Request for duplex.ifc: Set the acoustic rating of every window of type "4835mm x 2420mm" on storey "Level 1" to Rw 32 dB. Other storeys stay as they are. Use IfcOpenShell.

First a look at what the model holds.

```python
import ifcopenshell
import ifcopenshell.util.element

model = ifcopenshell.open("duplex.ifc")
print(model.schema)
storey = next(s for s in model.by_type("IfcBuildingStorey") if s.Name == "Level 1")
windows = [e for e in ifcopenshell.util.element.get_decomposition(storey) if e.is_a("IfcWindow")]
seen = {}
for e in windows:
    element_type = ifcopenshell.util.element.get_type(e)
    key = (element_type.Name if element_type != e and element_type else None, ifcopenshell.util.element.get_pset(e, "Pset_WindowCommon", "AcousticRating"))
    seen[key] = seen.get(key, 0) + 1
for (name, value), count in sorted(seen.items(), key=str):
    print(count, "x", name, "|", value)
```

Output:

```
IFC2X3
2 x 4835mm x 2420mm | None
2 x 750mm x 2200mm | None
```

```python
import ifcopenshell
import ifcopenshell.api.pset
import ifcopenshell.util.element

model = ifcopenshell.open("duplex.ifc")

storey = next(s for s in model.by_type("IfcBuildingStorey") if s.Name == "Level 1")
windows = [e for e in ifcopenshell.util.element.get_decomposition(storey) if e.is_a("IfcWindow")]

count = 0
for e in windows:
    element_type = ifcopenshell.util.element.get_type(e)
    if element_type in (None, e) or element_type.Name != "4835mm x 2420mm":
        continue
    # add_pset returns the element's existing set when there is one.
    pset = ifcopenshell.api.pset.add_pset(model, product=e, name="Pset_WindowCommon")
    ifcopenshell.api.pset.edit_pset(model, pset=pset, properties={"AcousticRating": "Rw 32 dB"})
    count += 1

print(count, "windows updated")

model.write("duplex_v2.ifc")
```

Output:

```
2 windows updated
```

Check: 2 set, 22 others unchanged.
